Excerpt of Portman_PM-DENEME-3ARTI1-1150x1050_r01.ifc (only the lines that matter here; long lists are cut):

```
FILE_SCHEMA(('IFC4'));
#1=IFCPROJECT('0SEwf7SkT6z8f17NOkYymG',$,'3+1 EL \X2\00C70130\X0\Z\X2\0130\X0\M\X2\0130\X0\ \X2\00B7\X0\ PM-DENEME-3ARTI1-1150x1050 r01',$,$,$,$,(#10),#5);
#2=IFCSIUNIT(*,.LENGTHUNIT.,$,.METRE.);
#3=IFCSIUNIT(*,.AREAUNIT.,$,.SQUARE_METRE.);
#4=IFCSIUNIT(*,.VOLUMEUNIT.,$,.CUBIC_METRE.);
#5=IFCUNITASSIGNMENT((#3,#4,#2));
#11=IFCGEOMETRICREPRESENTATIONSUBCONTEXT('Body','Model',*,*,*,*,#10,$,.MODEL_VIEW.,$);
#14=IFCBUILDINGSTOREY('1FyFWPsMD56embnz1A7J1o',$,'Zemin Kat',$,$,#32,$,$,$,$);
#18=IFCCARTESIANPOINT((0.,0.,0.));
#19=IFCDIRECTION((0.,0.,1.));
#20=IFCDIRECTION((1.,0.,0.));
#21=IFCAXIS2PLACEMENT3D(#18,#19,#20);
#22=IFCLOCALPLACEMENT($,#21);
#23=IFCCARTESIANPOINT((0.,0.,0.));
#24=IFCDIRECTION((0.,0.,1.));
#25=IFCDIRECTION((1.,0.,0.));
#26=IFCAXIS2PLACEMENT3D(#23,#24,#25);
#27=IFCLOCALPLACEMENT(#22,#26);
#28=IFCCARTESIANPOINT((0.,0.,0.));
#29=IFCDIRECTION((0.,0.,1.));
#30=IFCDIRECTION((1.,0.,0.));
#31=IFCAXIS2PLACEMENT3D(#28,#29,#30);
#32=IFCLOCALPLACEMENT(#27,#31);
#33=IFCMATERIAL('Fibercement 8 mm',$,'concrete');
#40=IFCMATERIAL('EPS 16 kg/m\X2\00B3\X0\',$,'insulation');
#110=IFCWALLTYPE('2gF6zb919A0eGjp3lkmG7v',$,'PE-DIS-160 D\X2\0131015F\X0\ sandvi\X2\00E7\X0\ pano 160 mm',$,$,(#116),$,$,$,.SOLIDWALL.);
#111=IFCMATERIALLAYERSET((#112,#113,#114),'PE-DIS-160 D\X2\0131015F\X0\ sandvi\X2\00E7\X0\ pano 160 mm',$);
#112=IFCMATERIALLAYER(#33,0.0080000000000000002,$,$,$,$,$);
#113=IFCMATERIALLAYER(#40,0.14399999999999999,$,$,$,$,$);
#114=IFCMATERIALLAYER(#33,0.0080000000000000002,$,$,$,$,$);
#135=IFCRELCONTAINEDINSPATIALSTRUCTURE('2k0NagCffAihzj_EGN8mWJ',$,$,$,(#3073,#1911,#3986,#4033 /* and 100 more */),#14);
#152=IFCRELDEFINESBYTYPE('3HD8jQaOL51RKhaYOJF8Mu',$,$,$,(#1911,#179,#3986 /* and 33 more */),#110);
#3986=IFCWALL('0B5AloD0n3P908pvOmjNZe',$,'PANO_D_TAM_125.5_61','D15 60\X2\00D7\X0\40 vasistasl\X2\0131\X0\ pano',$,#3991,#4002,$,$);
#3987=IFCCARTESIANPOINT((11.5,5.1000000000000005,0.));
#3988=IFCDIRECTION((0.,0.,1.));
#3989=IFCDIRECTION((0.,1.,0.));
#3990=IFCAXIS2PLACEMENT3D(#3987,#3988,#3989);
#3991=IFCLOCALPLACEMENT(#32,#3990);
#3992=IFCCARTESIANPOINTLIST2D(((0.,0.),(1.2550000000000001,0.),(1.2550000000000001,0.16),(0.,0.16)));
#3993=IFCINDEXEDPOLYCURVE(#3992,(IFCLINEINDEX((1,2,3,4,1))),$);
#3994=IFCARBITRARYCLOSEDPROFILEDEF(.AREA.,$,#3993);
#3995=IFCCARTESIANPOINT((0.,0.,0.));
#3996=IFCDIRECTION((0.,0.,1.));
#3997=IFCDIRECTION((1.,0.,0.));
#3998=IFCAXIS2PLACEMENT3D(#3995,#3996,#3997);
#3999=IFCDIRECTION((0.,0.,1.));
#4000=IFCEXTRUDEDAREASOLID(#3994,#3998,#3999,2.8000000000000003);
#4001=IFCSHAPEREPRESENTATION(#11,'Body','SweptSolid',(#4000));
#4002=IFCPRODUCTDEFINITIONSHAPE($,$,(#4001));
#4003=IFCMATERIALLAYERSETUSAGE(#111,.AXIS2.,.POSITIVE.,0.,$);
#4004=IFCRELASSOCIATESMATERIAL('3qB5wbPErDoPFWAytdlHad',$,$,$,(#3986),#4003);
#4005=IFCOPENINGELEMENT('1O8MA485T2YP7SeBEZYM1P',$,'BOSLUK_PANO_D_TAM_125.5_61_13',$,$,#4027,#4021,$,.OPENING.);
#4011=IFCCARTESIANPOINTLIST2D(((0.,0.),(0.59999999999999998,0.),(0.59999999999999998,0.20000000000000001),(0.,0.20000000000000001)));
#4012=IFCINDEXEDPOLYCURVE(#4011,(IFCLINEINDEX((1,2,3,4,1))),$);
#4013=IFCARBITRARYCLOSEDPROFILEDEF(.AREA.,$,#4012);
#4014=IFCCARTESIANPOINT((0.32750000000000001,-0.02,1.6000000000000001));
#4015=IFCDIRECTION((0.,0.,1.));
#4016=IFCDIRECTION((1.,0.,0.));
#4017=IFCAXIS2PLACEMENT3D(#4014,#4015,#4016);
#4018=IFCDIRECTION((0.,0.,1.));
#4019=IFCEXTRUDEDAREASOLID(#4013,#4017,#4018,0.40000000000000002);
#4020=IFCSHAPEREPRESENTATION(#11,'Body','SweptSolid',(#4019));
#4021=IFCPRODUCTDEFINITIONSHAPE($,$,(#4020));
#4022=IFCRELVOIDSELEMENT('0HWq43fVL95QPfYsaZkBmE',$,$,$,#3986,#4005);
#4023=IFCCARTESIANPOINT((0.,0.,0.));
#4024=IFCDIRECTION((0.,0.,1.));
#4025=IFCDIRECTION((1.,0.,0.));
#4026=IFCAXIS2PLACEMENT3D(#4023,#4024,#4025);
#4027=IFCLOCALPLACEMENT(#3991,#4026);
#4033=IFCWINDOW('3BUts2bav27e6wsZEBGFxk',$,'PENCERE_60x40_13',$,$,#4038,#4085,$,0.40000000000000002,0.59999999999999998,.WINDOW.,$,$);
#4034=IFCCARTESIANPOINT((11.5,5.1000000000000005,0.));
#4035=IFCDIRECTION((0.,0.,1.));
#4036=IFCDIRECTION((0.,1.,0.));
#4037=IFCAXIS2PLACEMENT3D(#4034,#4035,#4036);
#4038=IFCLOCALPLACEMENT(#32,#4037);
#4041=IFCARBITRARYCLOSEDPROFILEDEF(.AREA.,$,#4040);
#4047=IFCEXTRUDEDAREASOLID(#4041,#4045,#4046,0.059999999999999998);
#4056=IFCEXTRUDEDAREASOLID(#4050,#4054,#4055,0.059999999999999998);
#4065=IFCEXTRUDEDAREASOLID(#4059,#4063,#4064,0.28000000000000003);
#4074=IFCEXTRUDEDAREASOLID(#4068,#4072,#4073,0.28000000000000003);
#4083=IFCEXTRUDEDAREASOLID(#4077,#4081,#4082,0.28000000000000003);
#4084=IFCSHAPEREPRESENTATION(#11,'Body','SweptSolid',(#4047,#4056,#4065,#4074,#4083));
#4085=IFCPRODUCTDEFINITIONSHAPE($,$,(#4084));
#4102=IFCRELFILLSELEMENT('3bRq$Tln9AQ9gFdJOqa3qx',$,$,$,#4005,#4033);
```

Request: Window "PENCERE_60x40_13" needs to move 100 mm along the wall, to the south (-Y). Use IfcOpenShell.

```python
import ifcopenshell
import ifcopenshell.api.geometry
import ifcopenshell.util.placement

model = ifcopenshell.open("Portman_PM-DENEME-3ARTI1-1150x1050_r01.ifc")

window = model.by_id(4033)
opening = window.FillsVoids[0].RelatingOpeningElement
wall = opening.VoidsElements[0].RelatingBuildingElement

wall_matrix = ifcopenshell.util.placement.get_local_placement(wall.ObjectPlacement)
shift = wall_matrix[:3, 0] * -0.1
before = ifcopenshell.util.placement.get_local_placement(window.ObjectPlacement)[:3, 3].copy()

# The window is not placed relative to its opening, so move both.
for product in (opening, window):
    matrix = ifcopenshell.util.placement.get_local_placement(product.ObjectPlacement)
    matrix[:3, 3] += shift
    ifcopenshell.api.geometry.edit_object_placement(model, product=product, matrix=matrix, is_si=False)

after = ifcopenshell.util.placement.get_local_placement(window.ObjectPlacement)[:3, 3]
print("window moved by", (after - before).round(3) + 0.0)

model.write("Portman_PM-DENEME-3ARTI1-1150x1050_r01_updated.ifc")
```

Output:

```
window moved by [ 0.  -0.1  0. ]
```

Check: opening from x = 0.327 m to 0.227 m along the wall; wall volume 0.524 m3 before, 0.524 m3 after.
